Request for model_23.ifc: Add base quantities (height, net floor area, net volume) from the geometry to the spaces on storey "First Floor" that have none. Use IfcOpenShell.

First a look at what the model holds.

```python
import ifcopenshell
import ifcopenshell.util.element
import ifcopenshell.util.unit

model = ifcopenshell.open("model_23.ifc")
print(model.schema)
for unit_type in ("LENGTHUNIT", "AREAUNIT", "VOLUMEUNIT"):
    print(unit_type, ifcopenshell.util.unit.calculate_unit_scale(model, unit_type))
storey = next(s for s in model.by_type("IfcBuildingStorey") if s.Name == "First Floor")
spaces = [e for e in ifcopenshell.util.element.get_decomposition(storey) if e.is_a("IfcSpace")]
for e in sorted(spaces, key=lambda e: e.id()):
    print(e.id(), e.is_a(), e.Name, list(ifcopenshell.util.element.get_psets(e, qtos_only=True)), sep=" | ")
```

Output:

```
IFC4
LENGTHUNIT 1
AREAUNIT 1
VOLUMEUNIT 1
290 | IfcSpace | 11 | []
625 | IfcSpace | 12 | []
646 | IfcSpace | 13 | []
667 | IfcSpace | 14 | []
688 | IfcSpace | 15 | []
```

```python
import ifcopenshell
import ifcopenshell.api.pset
import ifcopenshell.geom
import ifcopenshell.util.element
import ifcopenshell.util.shape
import ifcopenshell.util.unit

model = ifcopenshell.open("model_23.ifc")
unit_scale = ifcopenshell.util.unit.calculate_unit_scale(model)
area_scale = ifcopenshell.util.unit.calculate_unit_scale(model, "AREAUNIT")
volume_scale = ifcopenshell.util.unit.calculate_unit_scale(model, "VOLUMEUNIT")
settings = ifcopenshell.geom.settings()

storey = next(s for s in model.by_type("IfcBuildingStorey") if s.Name == "First Floor")
spaces = [e for e in ifcopenshell.util.element.get_decomposition(storey) if e.is_a("IfcSpace")]

for e in sorted(spaces, key=lambda e: e.id()):
    if ifcopenshell.util.element.get_psets(e, qtos_only=True, should_inherit=False):
        continue
    # Geometry comes back in metres, in the element's own axes.
    shape = ifcopenshell.geom.create_shape(settings, e)
    values = {
        "Height": ifcopenshell.util.shape.get_z(shape.geometry) / unit_scale,
        "NetFloorArea": ifcopenshell.util.shape.get_footprint_area(shape.geometry) / area_scale,
        "NetVolume": ifcopenshell.util.shape.get_volume(shape.geometry) / volume_scale,
    }
    qto = ifcopenshell.api.pset.add_qto(model, product=e, name="Qto_SpaceBaseQuantities")
    ifcopenshell.api.pset.edit_qto(model, qto=qto, properties=values)
    print(e.id(), {k: round(v, 3) for k, v in values.items()})

model.write("model_23_v2.ifc")
```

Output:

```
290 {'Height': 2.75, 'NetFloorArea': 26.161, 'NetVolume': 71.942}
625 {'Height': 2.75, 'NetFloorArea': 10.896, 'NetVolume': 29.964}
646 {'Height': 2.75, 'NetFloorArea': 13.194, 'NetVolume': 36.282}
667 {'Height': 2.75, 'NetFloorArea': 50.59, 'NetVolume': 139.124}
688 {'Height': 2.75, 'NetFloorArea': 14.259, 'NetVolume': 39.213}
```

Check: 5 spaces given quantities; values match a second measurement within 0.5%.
